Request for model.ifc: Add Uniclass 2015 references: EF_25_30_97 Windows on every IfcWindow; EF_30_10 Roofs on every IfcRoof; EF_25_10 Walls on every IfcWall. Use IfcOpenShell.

First a look at what the model holds.

```python
import ifcopenshell

model = ifcopenshell.open("model.ifc")
print(model.schema)
print("classifications:", [c.Name for c in model.by_type("IfcClassification")])
for ifc_class in ("IfcDoor", "IfcRoof", "IfcStair", "IfcWall", "IfcWindow"):
    print(ifc_class, len(model.by_type(ifc_class)))
```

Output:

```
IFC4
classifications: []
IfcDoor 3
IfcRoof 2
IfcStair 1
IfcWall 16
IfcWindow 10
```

```python
import ifcopenshell
import ifcopenshell.api.classification

model = ifcopenshell.open("model.ifc")

system = ifcopenshell.api.classification.add_classification(model, classification="Uniclass 2015")

codes = {
    "IfcWindow": ("EF_25_30_97", "Windows"),
    "IfcRoof": ("EF_30_10", "Roofs"),
    "IfcWall": ("EF_25_10", "Walls"),
}
for ifc_class, (code, name) in codes.items():
    products = model.by_type(ifc_class)
    ifcopenshell.api.classification.add_reference(
        model, products=products, classification=system, identification=code, name=name
    )
    print(code, len(products))

model.write("model_updated.ifc")
```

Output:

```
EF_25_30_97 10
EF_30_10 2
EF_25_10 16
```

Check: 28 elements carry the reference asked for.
